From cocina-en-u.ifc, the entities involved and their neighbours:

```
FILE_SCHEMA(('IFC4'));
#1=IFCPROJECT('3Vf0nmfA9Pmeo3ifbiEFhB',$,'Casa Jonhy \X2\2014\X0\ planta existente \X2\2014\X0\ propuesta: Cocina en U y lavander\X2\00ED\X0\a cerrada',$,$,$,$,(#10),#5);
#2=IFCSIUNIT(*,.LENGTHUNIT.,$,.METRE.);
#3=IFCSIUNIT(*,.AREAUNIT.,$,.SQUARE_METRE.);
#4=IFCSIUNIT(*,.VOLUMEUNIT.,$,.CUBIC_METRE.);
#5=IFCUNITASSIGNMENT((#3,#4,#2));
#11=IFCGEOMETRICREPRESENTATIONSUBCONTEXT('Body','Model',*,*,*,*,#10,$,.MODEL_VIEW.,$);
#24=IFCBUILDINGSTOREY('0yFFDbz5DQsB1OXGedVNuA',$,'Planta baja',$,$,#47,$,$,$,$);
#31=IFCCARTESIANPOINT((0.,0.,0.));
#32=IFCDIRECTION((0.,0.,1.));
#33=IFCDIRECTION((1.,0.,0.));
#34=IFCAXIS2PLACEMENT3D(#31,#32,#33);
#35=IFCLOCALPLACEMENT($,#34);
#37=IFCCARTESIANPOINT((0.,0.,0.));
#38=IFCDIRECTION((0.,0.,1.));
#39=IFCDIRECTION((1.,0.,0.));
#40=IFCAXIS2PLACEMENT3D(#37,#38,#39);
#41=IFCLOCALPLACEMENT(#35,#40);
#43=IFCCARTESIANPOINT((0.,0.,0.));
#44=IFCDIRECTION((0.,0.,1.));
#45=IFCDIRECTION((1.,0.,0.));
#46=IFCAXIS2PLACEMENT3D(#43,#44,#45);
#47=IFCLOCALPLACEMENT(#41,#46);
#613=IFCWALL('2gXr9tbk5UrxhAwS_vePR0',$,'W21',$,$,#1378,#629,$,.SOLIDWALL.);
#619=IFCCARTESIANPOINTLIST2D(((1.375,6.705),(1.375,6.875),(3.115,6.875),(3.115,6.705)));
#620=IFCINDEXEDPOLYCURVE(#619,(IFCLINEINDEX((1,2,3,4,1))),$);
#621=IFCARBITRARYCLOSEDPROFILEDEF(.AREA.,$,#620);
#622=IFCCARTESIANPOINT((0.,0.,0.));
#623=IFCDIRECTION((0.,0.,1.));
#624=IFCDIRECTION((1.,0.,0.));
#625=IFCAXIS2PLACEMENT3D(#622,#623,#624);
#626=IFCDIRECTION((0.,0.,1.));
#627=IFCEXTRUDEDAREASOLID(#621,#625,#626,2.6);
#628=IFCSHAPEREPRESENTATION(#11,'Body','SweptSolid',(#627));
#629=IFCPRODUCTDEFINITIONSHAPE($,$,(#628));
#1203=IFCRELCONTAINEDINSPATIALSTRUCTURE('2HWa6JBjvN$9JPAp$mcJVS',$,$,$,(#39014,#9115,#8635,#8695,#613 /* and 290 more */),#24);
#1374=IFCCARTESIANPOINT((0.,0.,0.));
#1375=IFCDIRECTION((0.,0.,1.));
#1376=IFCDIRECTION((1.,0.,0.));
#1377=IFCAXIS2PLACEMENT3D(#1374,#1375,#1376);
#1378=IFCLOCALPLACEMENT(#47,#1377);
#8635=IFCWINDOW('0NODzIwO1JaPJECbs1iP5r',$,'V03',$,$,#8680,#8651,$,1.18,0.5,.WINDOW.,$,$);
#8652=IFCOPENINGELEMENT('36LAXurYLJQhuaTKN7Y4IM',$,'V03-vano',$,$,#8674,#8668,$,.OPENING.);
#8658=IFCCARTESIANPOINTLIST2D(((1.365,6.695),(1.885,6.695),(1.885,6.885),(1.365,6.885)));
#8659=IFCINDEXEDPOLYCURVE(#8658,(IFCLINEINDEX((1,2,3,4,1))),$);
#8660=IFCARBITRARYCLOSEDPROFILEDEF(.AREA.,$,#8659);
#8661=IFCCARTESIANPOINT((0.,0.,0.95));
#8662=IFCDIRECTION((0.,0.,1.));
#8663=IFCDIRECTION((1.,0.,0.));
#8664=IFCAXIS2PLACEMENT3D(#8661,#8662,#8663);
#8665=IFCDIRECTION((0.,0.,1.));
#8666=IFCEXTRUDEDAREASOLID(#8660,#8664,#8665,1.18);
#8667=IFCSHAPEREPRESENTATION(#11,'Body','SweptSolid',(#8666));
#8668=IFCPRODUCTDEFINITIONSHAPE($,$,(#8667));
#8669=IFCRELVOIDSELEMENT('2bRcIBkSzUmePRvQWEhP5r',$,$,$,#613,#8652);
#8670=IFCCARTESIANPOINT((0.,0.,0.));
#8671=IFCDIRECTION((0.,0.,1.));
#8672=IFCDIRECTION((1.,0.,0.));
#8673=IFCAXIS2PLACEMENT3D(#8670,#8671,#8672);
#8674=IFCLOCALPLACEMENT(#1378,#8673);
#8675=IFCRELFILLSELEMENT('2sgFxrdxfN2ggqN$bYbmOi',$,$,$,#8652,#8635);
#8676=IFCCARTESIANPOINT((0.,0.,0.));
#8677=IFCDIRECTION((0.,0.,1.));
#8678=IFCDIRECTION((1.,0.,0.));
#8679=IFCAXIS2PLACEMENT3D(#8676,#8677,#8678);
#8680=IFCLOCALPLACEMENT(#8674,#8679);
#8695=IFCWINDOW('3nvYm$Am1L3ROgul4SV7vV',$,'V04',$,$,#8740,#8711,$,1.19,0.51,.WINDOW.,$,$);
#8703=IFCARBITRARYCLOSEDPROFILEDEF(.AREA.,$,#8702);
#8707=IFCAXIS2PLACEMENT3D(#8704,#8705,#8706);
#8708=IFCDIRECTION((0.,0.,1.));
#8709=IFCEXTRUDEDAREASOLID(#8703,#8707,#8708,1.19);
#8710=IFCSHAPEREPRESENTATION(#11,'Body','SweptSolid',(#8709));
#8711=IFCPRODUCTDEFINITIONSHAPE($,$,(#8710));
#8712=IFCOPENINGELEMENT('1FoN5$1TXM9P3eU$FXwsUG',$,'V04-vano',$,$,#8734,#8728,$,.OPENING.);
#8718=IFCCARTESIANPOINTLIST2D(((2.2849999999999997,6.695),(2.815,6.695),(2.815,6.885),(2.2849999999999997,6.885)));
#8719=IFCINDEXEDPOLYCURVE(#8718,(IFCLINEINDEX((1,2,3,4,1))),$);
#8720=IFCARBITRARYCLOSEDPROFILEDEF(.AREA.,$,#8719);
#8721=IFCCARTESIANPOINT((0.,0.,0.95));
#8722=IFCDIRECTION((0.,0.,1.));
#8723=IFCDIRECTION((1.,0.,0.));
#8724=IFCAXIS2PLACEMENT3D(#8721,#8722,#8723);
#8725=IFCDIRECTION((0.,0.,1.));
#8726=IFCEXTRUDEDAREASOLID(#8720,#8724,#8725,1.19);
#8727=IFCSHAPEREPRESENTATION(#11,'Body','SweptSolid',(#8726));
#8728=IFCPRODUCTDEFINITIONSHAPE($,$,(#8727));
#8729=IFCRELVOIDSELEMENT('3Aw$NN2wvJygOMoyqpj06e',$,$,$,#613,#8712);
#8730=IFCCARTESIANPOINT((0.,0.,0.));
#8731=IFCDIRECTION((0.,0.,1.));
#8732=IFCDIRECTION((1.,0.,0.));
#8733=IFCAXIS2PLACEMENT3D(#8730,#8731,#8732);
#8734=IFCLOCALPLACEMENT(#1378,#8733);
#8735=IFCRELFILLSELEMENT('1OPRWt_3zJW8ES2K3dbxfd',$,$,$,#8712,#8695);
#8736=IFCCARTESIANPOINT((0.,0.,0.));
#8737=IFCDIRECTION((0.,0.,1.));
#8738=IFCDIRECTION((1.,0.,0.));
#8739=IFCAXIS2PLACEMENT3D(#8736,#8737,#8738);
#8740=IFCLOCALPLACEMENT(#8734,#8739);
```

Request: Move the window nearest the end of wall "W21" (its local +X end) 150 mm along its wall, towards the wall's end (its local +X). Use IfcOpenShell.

```python
import ifcopenshell
import ifcopenshell.api.geometry
import ifcopenshell.util.placement

model = ifcopenshell.open("cocina-en-u.ifc")

window = model.by_id(8695)
opening = window.FillsVoids[0].RelatingOpeningElement
wall = opening.VoidsElements[0].RelatingBuildingElement

wall_matrix = ifcopenshell.util.placement.get_local_placement(wall.ObjectPlacement)
shift = wall_matrix[:3, 0] * 0.15
before = ifcopenshell.util.placement.get_local_placement(window.ObjectPlacement)[:3, 3].copy()

# The window is placed relative to its opening, so it follows when the opening moves.
matrix = ifcopenshell.util.placement.get_local_placement(opening.ObjectPlacement)
matrix[:3, 3] += shift
ifcopenshell.api.geometry.edit_object_placement(
    model, product=opening, matrix=matrix, is_si=False, should_transform_children=True
)

after = ifcopenshell.util.placement.get_local_placement(window.ObjectPlacement)[:3, 3]
print("window moved by", (after - before).round(3) + 0.0)

model.write("cocina-en-u_edited.ifc")
```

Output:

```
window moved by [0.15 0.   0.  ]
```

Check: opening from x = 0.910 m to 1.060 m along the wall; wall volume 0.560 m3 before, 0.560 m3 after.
